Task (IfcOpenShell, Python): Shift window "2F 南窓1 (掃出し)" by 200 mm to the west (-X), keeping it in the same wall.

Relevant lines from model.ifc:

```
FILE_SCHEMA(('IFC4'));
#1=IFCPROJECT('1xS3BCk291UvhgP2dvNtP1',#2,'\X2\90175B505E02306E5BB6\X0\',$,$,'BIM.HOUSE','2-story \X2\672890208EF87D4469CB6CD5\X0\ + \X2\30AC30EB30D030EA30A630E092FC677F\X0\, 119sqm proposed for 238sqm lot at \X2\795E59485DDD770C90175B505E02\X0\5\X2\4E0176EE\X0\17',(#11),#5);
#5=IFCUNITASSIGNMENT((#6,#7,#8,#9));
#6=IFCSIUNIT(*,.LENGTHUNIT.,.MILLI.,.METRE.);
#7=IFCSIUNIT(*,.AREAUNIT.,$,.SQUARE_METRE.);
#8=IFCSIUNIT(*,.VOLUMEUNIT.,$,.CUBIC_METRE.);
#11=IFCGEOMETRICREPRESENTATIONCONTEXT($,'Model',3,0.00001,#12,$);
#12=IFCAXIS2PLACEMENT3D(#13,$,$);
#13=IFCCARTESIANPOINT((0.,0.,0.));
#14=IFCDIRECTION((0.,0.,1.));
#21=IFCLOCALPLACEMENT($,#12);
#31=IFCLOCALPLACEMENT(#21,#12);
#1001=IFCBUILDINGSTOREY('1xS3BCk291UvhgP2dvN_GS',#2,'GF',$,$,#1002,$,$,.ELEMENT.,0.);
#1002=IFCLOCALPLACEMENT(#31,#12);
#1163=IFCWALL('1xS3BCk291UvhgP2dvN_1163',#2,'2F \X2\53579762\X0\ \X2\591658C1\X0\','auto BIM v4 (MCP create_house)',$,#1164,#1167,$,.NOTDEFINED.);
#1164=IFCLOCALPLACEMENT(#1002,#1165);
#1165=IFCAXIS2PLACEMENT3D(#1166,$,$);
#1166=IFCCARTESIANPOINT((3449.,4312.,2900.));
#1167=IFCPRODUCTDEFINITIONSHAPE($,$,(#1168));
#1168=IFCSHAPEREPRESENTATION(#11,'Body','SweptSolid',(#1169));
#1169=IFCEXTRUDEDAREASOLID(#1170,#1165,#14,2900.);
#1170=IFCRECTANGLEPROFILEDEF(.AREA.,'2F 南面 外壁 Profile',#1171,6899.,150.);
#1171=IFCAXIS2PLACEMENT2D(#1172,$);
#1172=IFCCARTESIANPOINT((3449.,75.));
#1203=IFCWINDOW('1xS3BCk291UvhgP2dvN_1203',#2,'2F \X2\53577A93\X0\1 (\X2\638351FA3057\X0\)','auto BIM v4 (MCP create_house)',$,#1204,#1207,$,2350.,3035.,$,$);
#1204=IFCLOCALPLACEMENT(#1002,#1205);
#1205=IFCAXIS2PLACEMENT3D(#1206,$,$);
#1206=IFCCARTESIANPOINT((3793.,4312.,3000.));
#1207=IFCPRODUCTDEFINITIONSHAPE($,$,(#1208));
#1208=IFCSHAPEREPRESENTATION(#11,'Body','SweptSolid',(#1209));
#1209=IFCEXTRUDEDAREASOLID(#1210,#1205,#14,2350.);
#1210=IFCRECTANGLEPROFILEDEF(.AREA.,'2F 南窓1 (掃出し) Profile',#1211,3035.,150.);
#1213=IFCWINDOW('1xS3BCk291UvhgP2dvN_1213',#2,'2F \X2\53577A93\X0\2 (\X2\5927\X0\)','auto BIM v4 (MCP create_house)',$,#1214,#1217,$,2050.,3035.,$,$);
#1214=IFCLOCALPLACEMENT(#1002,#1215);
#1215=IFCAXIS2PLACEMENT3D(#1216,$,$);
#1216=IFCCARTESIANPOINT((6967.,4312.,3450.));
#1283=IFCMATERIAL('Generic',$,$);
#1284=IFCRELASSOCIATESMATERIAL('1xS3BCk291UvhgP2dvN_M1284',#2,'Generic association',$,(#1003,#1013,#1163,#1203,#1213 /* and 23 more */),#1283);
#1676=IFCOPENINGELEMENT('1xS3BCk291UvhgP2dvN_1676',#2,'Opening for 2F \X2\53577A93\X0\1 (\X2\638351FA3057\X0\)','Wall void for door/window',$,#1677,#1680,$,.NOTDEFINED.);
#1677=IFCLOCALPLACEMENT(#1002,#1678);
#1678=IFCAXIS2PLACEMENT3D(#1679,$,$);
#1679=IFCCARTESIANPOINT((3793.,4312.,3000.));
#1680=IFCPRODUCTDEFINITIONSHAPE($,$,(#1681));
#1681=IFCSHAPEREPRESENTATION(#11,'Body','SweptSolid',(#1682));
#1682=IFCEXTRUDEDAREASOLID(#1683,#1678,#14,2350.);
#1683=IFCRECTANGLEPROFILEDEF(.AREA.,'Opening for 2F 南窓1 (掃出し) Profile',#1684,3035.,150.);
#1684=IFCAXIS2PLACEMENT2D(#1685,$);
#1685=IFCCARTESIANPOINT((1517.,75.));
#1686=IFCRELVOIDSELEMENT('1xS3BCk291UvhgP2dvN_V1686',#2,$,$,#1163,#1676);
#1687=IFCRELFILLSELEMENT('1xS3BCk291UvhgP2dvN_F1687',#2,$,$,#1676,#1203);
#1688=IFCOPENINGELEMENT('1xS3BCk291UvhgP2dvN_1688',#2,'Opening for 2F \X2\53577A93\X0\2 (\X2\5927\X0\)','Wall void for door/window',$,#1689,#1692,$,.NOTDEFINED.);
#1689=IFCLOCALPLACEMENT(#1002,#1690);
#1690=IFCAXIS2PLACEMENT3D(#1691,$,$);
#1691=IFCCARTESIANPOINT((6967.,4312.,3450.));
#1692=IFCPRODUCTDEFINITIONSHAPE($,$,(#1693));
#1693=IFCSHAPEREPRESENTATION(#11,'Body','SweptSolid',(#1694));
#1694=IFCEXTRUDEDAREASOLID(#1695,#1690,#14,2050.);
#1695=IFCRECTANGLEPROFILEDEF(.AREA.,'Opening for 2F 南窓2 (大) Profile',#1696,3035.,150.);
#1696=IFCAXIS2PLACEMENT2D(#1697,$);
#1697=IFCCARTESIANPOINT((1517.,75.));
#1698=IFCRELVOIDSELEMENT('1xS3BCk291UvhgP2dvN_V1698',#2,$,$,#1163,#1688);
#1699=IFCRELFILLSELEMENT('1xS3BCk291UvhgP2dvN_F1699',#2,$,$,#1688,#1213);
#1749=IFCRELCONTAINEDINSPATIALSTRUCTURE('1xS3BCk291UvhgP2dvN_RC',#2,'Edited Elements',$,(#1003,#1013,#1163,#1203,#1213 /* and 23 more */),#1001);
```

```python
import ifcopenshell
import ifcopenshell.api.geometry
import ifcopenshell.util.placement
import ifcopenshell.util.unit

model = ifcopenshell.open("model.ifc")
unit_scale = ifcopenshell.util.unit.calculate_unit_scale(model)

window = model.by_guid("1xS3BCk291UvhgP2dvN_1203")
opening = window.FillsVoids[0].RelatingOpeningElement
wall = opening.VoidsElements[0].RelatingBuildingElement

wall_matrix = ifcopenshell.util.placement.get_local_placement(wall.ObjectPlacement)
shift = wall_matrix[:3, 0] * -0.2 / unit_scale
before = ifcopenshell.util.placement.get_local_placement(window.ObjectPlacement)[:3, 3].copy()

# The window is not placed relative to its opening, so move both.
for product in (opening, window):
    matrix = ifcopenshell.util.placement.get_local_placement(product.ObjectPlacement)
    matrix[:3, 3] += shift
    ifcopenshell.api.geometry.edit_object_placement(model, product=product, matrix=matrix, is_si=False)

after = ifcopenshell.util.placement.get_local_placement(window.ObjectPlacement)[:3, 3]
print("window moved by", (after - before).round(3) + 0.0)

model.write("model_edited.ifc")
```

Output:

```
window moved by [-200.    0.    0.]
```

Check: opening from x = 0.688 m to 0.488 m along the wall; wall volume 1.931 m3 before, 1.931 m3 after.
